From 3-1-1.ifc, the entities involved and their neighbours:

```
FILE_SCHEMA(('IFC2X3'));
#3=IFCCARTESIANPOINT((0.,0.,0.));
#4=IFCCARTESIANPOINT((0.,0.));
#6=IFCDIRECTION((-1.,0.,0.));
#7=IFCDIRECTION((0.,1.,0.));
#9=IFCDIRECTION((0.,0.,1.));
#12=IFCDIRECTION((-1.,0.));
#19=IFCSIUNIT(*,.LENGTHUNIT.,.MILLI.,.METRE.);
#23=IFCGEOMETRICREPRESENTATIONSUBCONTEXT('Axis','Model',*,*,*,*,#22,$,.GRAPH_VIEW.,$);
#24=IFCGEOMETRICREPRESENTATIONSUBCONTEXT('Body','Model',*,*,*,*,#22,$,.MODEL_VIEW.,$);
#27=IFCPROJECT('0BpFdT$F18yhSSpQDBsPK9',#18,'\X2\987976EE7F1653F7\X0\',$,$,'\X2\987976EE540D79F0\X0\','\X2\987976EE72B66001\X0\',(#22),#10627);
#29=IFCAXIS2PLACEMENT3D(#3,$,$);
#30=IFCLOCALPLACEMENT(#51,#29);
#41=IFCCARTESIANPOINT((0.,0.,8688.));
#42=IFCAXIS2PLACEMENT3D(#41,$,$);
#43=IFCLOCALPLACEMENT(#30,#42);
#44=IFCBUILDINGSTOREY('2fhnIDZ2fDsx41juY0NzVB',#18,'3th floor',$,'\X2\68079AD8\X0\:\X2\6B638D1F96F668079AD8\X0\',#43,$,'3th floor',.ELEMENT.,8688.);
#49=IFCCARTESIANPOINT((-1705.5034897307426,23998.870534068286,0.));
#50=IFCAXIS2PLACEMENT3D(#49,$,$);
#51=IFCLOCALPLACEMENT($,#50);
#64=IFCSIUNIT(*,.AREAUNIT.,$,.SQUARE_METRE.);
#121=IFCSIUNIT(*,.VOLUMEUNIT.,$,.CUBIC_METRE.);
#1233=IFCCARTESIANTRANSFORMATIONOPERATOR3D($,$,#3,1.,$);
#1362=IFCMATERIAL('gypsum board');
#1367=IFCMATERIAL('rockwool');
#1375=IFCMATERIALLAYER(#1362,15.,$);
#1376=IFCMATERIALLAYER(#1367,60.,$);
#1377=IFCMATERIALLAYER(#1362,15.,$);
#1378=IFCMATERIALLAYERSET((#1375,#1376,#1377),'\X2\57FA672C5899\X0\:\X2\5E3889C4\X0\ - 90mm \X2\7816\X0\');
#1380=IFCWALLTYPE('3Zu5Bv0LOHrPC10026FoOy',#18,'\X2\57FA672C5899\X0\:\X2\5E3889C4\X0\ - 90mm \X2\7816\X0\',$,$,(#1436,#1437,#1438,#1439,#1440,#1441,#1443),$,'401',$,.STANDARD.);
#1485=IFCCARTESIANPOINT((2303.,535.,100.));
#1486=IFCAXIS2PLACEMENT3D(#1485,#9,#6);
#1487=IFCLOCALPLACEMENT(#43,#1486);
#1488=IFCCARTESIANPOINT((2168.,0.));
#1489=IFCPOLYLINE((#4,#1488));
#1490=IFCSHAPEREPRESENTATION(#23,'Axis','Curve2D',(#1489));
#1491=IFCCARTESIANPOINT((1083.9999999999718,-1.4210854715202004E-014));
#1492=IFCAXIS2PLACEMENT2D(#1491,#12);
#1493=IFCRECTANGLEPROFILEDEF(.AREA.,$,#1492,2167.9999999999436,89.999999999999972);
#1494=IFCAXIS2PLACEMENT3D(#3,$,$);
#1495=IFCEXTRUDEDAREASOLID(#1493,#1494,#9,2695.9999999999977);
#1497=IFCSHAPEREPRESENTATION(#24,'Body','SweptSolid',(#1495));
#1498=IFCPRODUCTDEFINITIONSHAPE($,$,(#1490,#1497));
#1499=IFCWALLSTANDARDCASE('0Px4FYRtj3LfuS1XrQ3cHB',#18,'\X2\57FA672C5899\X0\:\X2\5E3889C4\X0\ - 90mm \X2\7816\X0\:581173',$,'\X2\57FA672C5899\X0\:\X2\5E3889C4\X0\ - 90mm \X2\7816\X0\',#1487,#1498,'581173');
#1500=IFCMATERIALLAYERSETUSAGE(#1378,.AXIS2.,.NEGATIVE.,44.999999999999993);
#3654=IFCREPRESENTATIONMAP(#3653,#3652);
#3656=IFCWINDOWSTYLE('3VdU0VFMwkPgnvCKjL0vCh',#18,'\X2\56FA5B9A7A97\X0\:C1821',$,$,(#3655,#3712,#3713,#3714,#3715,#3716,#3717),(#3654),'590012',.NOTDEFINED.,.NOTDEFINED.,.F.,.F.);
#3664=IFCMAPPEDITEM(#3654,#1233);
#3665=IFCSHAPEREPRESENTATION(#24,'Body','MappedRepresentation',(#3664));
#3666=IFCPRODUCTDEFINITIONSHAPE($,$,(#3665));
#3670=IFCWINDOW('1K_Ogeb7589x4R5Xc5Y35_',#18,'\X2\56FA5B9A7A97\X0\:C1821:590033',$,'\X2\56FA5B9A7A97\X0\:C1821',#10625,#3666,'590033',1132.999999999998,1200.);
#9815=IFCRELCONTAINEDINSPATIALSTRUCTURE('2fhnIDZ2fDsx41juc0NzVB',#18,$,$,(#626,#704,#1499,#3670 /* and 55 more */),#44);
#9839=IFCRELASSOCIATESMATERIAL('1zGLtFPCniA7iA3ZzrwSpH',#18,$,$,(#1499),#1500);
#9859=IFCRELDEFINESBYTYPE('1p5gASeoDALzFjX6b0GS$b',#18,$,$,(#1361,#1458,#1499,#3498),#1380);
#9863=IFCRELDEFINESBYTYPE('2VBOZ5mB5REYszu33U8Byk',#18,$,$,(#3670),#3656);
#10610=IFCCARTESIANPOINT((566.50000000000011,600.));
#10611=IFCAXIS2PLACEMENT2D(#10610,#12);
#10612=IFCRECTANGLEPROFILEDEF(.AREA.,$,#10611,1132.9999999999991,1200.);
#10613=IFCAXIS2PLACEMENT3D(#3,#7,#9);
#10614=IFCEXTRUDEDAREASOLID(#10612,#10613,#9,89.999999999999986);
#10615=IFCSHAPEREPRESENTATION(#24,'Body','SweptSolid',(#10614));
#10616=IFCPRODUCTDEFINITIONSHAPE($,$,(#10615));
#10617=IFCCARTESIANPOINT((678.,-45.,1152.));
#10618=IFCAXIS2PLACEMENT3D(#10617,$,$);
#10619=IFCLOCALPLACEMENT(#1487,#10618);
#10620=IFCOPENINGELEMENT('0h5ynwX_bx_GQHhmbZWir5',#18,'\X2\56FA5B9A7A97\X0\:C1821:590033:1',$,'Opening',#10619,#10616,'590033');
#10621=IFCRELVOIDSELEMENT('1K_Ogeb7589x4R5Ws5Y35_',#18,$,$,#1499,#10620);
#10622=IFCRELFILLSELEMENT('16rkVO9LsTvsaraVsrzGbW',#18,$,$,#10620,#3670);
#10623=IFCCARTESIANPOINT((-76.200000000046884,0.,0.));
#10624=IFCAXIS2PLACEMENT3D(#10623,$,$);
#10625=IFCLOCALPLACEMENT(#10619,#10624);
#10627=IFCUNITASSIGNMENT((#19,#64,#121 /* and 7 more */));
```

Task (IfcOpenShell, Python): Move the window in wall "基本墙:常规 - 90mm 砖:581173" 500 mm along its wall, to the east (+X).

```python
import ifcopenshell
import ifcopenshell.api.geometry
import ifcopenshell.util.placement

model = ifcopenshell.open("3-1-1.ifc")

window = model.by_guid("1K_Ogeb7589x4R5Xc5Y35_")
opening = window.FillsVoids[0].RelatingOpeningElement
wall = opening.VoidsElements[0].RelatingBuildingElement

wall_matrix = ifcopenshell.util.placement.get_local_placement(wall.ObjectPlacement)
shift = wall_matrix[:3, 0] * -500.0
before = ifcopenshell.util.placement.get_local_placement(window.ObjectPlacement)[:3, 3].copy()

# The window is placed relative to its opening, so it follows when the opening moves.
matrix = ifcopenshell.util.placement.get_local_placement(opening.ObjectPlacement)
matrix[:3, 3] += shift
ifcopenshell.api.geometry.edit_object_placement(
    model, product=opening, matrix=matrix, is_si=False, should_transform_children=True
)

after = ifcopenshell.util.placement.get_local_placement(window.ObjectPlacement)[:3, 3]
print("window moved by", (after - before).round(3) + 0.0)

model.write("3-1-1_edited.ifc")
```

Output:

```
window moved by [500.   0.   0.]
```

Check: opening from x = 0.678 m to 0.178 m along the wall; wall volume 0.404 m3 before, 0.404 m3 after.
